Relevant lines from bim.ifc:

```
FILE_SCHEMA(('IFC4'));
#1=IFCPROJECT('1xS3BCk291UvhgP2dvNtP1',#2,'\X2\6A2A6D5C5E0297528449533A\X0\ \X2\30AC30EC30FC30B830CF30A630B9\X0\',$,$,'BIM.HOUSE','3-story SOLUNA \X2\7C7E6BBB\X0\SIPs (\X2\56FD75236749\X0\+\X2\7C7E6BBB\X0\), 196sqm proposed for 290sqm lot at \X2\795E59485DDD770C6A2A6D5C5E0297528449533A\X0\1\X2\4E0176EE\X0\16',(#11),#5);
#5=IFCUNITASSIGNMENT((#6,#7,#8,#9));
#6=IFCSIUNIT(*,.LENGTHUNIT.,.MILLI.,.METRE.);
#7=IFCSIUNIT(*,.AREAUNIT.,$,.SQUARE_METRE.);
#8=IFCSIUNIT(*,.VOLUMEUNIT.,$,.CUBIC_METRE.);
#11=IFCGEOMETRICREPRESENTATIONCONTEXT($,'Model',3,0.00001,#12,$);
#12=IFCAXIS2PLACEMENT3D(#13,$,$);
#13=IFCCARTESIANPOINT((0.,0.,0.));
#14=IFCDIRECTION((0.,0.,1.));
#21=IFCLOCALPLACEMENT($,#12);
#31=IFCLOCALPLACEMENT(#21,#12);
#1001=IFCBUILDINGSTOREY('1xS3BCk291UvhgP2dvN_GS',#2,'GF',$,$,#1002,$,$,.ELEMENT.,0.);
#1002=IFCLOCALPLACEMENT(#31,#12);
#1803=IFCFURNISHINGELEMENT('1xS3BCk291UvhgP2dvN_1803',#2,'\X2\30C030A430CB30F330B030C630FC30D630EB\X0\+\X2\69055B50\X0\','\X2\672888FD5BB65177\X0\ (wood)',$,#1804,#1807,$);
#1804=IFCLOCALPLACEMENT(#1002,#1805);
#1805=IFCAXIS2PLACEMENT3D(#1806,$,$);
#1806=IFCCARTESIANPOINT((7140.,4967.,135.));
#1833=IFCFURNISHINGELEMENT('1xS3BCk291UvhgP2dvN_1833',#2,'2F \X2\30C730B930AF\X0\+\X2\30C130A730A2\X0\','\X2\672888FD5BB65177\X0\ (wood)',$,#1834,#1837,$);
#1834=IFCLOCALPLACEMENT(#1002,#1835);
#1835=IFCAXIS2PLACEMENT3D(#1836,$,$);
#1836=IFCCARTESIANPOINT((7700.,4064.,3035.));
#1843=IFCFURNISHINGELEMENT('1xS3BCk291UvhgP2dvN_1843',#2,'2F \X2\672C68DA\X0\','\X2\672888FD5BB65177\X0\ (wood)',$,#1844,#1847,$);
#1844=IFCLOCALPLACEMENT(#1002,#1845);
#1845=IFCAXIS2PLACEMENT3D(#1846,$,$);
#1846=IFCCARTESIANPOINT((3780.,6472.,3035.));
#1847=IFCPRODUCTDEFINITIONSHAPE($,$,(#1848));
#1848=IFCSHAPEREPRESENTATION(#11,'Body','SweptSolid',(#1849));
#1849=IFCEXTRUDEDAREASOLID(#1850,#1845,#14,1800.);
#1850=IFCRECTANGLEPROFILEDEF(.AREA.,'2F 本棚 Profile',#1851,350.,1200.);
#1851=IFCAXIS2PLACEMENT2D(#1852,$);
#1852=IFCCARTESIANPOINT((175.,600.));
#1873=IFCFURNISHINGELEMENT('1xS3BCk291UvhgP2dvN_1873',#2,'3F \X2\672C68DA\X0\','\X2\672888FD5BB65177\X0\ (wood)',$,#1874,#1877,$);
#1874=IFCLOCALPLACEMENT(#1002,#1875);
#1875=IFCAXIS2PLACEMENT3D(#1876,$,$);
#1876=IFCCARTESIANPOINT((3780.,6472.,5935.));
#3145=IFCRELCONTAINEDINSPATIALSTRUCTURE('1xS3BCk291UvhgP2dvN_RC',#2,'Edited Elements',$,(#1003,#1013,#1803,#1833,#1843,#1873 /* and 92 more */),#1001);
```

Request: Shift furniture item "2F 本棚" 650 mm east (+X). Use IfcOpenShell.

```python
import ifcopenshell
import ifcopenshell.api.geometry
import ifcopenshell.util.placement
import ifcopenshell.util.unit

model = ifcopenshell.open("bim.ifc")
unit_scale = ifcopenshell.util.unit.calculate_unit_scale(model)

item = model.by_guid("1xS3BCk291UvhgP2dvN_1843")
matrix = ifcopenshell.util.placement.get_local_placement(item.ObjectPlacement)
matrix[0, 3] += 0.65 / unit_scale
ifcopenshell.api.geometry.edit_object_placement(model, product=item, matrix=matrix, is_si=False)

print(ifcopenshell.util.placement.get_local_placement(item.ObjectPlacement).round(3) + 0.0)

model.write("bim_edited.ifc")
```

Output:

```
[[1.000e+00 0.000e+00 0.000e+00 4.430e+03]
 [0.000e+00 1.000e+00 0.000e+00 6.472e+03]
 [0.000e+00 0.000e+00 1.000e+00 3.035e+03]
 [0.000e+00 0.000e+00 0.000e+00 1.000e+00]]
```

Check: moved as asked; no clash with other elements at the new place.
